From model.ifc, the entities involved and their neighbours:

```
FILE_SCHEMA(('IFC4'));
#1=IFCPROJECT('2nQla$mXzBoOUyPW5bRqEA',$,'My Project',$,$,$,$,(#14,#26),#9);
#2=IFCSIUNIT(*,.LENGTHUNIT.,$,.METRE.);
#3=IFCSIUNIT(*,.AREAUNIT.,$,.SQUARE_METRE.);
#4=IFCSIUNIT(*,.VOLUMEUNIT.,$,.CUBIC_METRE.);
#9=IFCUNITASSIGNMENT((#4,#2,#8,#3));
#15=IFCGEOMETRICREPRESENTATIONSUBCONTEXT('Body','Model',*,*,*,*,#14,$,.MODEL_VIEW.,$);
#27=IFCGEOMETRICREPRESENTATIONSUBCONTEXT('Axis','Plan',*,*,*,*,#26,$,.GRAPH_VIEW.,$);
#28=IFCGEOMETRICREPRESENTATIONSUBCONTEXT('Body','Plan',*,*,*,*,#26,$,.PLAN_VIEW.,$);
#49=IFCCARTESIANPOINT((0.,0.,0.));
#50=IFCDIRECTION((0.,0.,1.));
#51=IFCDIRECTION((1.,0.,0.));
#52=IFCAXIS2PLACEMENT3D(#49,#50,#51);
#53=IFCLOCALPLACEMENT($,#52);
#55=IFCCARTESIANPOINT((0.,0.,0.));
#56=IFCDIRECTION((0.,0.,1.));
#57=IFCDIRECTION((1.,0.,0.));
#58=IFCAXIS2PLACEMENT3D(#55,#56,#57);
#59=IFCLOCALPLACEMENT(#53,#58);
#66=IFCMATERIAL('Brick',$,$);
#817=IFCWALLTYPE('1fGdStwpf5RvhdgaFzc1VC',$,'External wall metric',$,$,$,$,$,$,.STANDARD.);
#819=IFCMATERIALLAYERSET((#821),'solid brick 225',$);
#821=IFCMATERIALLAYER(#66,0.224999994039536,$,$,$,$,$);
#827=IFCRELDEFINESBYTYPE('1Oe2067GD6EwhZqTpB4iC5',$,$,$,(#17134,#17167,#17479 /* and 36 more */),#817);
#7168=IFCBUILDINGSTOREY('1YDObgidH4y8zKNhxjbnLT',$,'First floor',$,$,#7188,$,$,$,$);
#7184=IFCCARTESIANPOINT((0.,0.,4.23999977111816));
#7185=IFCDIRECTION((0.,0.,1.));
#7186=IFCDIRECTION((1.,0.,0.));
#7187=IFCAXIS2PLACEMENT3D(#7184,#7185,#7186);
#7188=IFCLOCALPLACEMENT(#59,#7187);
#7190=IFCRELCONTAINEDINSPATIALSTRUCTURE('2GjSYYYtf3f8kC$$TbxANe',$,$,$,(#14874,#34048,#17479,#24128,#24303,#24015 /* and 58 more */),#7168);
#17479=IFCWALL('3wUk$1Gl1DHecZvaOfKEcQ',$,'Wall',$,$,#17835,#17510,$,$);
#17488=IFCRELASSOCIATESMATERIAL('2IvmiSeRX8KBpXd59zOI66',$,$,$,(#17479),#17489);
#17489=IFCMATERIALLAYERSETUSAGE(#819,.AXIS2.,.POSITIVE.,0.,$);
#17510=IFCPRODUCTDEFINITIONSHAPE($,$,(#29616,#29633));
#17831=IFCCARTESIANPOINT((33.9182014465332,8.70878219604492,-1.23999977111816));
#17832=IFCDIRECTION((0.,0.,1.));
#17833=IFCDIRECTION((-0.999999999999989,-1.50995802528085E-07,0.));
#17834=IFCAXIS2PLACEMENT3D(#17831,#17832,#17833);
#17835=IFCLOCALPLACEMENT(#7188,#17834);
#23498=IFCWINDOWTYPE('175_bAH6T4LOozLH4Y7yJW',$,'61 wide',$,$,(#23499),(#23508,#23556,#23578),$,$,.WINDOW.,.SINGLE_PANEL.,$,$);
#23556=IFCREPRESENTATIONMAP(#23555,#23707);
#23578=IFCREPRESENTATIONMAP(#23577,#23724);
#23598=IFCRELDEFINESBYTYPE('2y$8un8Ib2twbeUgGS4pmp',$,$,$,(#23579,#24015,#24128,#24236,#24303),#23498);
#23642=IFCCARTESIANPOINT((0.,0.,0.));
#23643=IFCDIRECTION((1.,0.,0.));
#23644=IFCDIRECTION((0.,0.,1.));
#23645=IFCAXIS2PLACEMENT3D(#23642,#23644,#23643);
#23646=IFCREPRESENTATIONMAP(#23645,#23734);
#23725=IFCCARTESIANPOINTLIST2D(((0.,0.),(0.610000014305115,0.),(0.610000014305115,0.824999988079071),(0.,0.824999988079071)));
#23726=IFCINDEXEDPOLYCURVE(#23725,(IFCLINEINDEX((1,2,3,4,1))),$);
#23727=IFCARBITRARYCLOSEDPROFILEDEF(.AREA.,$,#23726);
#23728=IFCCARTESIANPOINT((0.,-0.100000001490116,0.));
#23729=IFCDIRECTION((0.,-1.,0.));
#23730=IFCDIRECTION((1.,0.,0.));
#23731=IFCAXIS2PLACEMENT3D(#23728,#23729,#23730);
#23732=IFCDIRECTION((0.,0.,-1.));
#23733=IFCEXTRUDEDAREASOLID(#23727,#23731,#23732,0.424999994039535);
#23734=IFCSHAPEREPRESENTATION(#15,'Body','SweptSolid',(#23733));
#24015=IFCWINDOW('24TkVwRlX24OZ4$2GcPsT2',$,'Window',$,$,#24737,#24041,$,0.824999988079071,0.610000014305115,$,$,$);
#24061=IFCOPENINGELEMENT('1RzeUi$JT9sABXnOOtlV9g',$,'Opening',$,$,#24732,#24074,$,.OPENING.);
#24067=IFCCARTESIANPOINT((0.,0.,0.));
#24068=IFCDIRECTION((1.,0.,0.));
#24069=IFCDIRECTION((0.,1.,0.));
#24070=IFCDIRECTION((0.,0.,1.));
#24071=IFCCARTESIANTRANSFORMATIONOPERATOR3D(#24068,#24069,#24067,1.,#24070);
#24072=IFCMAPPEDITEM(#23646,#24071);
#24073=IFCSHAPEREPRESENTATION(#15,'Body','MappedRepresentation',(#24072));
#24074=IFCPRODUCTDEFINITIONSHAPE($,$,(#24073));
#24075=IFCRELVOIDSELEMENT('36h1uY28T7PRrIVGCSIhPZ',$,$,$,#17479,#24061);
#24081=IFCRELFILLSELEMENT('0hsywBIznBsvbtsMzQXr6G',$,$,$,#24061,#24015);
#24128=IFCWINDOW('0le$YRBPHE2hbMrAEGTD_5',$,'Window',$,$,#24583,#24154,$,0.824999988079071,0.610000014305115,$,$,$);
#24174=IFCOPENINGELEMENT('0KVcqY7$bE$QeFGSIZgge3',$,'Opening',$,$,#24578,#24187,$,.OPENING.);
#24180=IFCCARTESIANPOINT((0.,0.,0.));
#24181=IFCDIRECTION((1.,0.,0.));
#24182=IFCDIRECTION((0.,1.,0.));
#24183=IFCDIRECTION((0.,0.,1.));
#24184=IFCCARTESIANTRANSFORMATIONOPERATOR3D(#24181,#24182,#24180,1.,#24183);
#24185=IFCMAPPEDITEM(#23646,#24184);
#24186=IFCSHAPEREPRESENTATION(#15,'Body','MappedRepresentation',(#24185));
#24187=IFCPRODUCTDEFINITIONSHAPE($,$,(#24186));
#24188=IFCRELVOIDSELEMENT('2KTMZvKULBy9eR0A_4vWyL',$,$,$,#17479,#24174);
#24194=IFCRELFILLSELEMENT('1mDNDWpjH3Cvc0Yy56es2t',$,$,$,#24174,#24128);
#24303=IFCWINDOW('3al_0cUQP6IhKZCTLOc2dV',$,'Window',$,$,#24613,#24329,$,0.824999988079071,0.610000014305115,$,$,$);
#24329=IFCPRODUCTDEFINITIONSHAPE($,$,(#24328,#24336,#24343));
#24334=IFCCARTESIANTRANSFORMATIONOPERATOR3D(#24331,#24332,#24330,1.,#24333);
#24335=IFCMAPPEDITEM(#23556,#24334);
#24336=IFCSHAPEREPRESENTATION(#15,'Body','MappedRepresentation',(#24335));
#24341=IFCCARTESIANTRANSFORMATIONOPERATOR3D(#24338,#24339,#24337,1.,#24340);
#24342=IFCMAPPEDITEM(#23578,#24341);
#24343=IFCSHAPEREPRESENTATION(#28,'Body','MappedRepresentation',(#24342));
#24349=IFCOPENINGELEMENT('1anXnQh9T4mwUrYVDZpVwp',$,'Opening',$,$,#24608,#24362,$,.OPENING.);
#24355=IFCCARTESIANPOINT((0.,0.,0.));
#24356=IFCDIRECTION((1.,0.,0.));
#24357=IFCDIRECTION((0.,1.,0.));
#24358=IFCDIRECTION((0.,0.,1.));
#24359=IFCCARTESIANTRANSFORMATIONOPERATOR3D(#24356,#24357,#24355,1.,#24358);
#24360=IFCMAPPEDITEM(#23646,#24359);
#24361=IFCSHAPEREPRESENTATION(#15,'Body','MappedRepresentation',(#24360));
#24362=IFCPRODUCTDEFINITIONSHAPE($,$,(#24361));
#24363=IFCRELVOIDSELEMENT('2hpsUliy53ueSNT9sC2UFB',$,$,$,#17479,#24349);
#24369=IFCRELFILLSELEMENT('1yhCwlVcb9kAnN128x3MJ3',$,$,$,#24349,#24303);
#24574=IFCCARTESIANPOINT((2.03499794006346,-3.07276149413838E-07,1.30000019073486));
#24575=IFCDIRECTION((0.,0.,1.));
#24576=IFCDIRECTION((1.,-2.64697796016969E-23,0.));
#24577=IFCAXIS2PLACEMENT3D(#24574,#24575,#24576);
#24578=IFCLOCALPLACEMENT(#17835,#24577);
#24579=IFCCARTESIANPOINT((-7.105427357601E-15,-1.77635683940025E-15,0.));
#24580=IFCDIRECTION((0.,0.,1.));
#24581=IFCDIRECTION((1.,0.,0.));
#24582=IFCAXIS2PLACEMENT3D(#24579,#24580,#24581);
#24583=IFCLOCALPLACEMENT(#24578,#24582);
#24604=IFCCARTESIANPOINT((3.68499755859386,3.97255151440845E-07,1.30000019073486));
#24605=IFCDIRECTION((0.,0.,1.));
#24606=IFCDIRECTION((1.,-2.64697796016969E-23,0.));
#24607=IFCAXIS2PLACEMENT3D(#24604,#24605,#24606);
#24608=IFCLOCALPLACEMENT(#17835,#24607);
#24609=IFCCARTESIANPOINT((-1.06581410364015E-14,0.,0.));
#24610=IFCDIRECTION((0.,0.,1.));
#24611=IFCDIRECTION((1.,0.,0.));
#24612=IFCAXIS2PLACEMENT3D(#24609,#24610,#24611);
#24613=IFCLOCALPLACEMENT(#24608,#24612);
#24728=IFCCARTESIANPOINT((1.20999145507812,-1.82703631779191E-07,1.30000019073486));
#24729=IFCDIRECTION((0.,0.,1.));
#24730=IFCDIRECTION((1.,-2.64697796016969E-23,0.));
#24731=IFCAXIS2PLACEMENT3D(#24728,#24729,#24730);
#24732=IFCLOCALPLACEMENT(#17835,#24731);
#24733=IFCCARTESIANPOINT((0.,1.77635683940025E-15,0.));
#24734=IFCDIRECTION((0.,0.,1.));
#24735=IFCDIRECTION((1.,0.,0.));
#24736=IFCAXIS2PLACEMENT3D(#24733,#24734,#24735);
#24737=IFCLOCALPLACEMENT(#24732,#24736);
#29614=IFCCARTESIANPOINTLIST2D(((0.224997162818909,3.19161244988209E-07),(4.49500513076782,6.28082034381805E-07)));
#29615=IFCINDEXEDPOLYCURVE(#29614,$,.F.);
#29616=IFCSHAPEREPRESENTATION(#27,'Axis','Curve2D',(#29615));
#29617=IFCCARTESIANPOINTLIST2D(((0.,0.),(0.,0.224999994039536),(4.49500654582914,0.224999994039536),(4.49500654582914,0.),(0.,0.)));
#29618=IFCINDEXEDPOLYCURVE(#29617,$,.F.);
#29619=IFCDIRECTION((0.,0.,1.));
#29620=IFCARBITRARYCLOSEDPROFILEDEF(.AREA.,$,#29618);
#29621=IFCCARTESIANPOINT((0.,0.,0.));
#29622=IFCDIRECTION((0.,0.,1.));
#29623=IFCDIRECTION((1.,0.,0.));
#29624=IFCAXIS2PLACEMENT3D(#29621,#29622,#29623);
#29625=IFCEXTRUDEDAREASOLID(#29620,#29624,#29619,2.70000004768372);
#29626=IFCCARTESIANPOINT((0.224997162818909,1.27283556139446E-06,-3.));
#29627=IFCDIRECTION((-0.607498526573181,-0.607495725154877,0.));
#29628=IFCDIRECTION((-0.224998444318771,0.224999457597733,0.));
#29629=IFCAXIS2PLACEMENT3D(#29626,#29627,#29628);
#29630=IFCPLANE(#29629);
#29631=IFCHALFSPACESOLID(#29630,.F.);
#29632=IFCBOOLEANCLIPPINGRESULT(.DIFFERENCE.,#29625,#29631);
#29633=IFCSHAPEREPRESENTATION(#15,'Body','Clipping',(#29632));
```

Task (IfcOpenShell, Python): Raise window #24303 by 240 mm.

```python
import numpy as np
import ifcopenshell
import ifcopenshell.api.geometry
import ifcopenshell.util.placement
import ifcopenshell.util.unit

model = ifcopenshell.open("model.ifc")
unit_scale = ifcopenshell.util.unit.calculate_unit_scale(model)

window = model.by_guid("3al_0cUQP6IhKZCTLOc2dV")
opening = window.FillsVoids[0].RelatingOpeningElement
dz = 0.24

shift = np.array([0.0, 0.0, dz])
# The window is placed relative to its opening, so it follows when the opening moves.
matrix = ifcopenshell.util.placement.get_local_placement(opening.ObjectPlacement)
matrix[:3, 3] += shift
ifcopenshell.api.geometry.edit_object_placement(
    model, product=opening, matrix=matrix, is_si=False, should_transform_children=True
)

print(f"moved by {dz * unit_scale:+.3f} m")

model.write("model_v2.ifc")
```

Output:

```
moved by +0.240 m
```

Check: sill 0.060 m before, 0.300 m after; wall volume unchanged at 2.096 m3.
